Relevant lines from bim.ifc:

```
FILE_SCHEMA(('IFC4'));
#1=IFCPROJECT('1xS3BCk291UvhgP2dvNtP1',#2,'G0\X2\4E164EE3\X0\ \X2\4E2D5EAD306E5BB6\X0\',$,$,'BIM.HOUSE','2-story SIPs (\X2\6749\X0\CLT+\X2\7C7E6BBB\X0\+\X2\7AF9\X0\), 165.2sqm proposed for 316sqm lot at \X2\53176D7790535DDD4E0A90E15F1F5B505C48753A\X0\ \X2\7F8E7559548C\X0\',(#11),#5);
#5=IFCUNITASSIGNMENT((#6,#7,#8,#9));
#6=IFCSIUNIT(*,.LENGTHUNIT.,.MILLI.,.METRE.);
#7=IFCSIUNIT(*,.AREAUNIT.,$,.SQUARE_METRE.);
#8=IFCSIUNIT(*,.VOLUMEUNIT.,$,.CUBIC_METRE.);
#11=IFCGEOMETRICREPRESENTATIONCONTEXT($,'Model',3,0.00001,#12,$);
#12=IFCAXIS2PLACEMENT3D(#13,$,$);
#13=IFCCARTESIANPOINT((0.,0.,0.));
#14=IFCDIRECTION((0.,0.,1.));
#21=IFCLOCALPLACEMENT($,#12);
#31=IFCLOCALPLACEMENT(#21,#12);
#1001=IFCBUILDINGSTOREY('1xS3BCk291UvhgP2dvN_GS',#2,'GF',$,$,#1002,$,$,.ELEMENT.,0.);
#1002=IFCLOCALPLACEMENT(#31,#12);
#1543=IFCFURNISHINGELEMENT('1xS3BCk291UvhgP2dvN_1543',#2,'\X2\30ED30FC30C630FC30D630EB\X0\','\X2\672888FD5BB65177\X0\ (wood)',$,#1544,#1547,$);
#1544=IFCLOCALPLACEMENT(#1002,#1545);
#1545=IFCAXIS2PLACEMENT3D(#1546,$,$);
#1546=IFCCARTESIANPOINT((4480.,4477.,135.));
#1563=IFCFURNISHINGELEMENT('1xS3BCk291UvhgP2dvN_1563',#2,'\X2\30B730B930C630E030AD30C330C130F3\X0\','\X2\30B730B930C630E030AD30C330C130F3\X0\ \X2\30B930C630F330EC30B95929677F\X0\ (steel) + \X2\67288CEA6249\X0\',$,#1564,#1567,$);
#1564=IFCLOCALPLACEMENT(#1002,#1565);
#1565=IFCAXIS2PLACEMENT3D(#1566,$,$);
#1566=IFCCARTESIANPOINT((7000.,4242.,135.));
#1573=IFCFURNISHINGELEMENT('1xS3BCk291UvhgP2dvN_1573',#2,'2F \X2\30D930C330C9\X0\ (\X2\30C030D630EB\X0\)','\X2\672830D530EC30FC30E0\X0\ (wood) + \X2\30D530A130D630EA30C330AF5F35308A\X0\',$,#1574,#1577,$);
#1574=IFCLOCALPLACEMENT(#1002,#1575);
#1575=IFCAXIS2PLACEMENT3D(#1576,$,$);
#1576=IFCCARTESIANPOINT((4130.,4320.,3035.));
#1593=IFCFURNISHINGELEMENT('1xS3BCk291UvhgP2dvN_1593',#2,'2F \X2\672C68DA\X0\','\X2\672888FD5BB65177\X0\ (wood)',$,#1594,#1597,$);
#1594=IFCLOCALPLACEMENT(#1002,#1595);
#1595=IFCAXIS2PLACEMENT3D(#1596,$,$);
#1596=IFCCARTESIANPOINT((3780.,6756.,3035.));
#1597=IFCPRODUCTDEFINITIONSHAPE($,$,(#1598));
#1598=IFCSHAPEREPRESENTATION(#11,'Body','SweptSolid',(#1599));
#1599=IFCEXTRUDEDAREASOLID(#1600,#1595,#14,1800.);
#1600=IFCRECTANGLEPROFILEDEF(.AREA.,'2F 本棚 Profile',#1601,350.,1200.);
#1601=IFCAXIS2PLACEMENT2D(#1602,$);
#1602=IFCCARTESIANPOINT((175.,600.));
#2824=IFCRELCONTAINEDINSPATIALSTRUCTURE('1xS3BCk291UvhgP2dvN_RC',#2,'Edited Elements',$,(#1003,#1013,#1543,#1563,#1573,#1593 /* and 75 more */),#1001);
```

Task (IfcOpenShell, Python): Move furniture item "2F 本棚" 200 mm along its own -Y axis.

```python
import ifcopenshell
import ifcopenshell.api.geometry
import ifcopenshell.util.placement
import ifcopenshell.util.unit

model = ifcopenshell.open("bim.ifc")
unit_scale = ifcopenshell.util.unit.calculate_unit_scale(model)

item = model.by_guid("1xS3BCk291UvhgP2dvN_1593")
matrix = ifcopenshell.util.placement.get_local_placement(item.ObjectPlacement)
matrix[:3, 3] -= matrix[:3, 1] * 0.2 / unit_scale
ifcopenshell.api.geometry.edit_object_placement(model, product=item, matrix=matrix, is_si=False)

print(ifcopenshell.util.placement.get_local_placement(item.ObjectPlacement).round(3) + 0.0)

model.write("bim_v2.ifc")
```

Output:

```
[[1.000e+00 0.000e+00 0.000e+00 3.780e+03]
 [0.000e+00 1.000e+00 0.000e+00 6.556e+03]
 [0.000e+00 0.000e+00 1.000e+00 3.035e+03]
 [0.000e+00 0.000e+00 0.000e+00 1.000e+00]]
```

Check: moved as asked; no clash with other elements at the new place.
